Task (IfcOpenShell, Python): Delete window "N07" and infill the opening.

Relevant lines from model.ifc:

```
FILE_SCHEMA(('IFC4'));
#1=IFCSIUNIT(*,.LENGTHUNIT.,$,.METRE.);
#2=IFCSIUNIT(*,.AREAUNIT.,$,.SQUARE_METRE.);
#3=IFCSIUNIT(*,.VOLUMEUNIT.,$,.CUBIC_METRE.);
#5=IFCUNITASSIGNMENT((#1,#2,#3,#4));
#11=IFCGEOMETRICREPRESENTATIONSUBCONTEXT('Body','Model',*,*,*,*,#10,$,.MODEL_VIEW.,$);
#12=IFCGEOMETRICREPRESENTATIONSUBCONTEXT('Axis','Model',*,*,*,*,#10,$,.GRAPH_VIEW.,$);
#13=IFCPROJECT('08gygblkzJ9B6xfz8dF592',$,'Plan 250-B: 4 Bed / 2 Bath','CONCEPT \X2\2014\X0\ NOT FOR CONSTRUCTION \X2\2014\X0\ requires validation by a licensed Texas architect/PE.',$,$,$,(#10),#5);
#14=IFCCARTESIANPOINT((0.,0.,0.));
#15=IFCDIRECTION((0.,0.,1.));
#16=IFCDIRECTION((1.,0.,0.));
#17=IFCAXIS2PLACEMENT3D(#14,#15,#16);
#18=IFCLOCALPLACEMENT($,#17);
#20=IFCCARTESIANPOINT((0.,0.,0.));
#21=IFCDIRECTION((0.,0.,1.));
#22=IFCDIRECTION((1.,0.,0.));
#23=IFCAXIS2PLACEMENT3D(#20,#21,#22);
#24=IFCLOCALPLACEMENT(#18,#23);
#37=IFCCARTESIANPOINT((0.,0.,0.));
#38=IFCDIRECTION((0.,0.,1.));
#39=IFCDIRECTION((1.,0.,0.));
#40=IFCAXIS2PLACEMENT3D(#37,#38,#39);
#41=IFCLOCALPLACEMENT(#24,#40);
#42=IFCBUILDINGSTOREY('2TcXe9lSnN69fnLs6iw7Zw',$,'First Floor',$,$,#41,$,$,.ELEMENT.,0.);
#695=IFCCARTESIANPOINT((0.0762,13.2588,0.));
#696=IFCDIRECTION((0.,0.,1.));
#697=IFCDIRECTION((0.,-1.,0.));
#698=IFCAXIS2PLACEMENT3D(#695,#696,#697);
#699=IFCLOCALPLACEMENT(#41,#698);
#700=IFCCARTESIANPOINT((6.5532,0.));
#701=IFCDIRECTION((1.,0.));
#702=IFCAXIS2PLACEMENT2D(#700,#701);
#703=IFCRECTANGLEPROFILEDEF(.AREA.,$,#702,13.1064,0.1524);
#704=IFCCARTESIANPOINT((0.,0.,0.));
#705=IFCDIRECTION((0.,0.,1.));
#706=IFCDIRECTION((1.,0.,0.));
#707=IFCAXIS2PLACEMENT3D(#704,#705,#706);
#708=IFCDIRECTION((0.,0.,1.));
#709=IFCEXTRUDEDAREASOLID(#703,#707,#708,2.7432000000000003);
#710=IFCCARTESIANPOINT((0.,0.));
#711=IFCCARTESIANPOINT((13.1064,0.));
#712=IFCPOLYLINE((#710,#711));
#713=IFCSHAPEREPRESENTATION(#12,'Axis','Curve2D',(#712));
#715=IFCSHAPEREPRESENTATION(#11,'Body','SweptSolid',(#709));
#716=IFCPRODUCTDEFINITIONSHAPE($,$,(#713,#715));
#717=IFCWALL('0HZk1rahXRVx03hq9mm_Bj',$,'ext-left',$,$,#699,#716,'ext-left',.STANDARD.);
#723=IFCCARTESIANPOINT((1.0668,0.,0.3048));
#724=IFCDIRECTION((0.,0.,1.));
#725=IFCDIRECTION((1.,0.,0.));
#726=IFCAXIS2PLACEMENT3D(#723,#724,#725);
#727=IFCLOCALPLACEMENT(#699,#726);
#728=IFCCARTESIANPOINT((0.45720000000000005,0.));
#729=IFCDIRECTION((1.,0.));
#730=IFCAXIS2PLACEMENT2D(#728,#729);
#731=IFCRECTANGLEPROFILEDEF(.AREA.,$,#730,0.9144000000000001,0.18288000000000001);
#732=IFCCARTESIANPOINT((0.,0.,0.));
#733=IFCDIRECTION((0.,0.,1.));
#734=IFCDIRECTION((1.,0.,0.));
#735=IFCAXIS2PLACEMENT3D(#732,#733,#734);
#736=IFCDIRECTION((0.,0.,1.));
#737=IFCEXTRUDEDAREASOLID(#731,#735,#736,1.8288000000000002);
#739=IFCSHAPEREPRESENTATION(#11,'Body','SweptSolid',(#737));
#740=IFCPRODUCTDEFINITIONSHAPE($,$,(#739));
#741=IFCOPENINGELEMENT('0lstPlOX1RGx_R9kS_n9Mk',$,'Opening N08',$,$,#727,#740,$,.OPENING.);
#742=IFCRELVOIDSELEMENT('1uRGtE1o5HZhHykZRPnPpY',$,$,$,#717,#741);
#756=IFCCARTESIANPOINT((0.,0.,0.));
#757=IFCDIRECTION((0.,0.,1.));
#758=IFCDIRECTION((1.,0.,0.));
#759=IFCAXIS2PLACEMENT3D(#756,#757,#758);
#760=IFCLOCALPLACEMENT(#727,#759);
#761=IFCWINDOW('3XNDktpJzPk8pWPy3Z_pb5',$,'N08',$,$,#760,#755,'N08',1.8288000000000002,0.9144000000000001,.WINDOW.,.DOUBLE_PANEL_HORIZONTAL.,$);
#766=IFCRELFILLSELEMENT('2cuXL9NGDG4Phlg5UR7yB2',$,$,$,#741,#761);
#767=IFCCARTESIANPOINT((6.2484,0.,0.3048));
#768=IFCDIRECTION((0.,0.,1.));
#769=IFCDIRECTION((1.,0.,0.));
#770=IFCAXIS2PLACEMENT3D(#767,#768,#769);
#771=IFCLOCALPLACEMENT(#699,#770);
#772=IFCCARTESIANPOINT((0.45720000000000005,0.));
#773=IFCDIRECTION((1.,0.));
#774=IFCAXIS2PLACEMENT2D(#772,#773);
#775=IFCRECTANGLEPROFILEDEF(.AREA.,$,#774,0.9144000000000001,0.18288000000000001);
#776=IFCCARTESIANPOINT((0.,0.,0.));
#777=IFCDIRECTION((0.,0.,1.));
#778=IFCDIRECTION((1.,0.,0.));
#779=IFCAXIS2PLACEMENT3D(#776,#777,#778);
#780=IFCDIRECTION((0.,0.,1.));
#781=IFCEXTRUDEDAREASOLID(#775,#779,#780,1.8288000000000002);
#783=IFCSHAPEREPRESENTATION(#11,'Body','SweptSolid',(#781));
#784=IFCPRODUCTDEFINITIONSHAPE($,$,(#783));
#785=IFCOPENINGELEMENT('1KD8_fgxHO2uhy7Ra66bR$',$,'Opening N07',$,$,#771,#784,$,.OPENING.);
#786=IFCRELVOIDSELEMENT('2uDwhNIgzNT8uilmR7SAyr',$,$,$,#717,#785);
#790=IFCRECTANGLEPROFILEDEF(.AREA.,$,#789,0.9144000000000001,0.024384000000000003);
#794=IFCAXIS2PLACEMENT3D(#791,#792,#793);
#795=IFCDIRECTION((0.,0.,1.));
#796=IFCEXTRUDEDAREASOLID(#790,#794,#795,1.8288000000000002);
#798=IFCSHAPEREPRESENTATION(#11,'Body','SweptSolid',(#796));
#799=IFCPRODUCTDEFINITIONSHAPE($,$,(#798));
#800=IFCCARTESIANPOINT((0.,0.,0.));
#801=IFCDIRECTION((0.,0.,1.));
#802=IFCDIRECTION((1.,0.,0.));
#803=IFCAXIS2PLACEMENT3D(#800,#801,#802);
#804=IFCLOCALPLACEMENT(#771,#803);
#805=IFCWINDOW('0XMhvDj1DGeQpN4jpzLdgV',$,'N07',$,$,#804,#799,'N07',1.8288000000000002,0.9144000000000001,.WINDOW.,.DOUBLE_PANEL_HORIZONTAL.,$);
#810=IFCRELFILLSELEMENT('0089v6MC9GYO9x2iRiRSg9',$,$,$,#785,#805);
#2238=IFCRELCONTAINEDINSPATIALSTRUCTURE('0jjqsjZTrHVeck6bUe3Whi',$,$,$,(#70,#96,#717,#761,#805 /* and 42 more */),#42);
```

```python
import ifcopenshell
import ifcopenshell.api.feature
import ifcopenshell.api.root
import ifcopenshell.geom
import ifcopenshell.util.shape

model = ifcopenshell.open("model.ifc")
settings = ifcopenshell.geom.settings()


def volume(element):
    """Net volume in cubic metres, openings subtracted."""
    shape = ifcopenshell.geom.create_shape(settings, element)
    return ifcopenshell.util.shape.get_volume(shape.geometry)


window = model.by_guid("0XMhvDj1DGeQpN4jpzLdgV")
opening = window.FillsVoids[0].RelatingOpeningElement
wall = opening.VoidsElements[0].RelatingBuildingElement
before = volume(wall)

ifcopenshell.api.root.remove_product(model, product=window)
ifcopenshell.api.feature.remove_feature(model, feature=opening)

after = volume(wall)

print(f"wall volume {before:.3f} -> {after:.3f} m3")

model.write("model_v2.ifc")
```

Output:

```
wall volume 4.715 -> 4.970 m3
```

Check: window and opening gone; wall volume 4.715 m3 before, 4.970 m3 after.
